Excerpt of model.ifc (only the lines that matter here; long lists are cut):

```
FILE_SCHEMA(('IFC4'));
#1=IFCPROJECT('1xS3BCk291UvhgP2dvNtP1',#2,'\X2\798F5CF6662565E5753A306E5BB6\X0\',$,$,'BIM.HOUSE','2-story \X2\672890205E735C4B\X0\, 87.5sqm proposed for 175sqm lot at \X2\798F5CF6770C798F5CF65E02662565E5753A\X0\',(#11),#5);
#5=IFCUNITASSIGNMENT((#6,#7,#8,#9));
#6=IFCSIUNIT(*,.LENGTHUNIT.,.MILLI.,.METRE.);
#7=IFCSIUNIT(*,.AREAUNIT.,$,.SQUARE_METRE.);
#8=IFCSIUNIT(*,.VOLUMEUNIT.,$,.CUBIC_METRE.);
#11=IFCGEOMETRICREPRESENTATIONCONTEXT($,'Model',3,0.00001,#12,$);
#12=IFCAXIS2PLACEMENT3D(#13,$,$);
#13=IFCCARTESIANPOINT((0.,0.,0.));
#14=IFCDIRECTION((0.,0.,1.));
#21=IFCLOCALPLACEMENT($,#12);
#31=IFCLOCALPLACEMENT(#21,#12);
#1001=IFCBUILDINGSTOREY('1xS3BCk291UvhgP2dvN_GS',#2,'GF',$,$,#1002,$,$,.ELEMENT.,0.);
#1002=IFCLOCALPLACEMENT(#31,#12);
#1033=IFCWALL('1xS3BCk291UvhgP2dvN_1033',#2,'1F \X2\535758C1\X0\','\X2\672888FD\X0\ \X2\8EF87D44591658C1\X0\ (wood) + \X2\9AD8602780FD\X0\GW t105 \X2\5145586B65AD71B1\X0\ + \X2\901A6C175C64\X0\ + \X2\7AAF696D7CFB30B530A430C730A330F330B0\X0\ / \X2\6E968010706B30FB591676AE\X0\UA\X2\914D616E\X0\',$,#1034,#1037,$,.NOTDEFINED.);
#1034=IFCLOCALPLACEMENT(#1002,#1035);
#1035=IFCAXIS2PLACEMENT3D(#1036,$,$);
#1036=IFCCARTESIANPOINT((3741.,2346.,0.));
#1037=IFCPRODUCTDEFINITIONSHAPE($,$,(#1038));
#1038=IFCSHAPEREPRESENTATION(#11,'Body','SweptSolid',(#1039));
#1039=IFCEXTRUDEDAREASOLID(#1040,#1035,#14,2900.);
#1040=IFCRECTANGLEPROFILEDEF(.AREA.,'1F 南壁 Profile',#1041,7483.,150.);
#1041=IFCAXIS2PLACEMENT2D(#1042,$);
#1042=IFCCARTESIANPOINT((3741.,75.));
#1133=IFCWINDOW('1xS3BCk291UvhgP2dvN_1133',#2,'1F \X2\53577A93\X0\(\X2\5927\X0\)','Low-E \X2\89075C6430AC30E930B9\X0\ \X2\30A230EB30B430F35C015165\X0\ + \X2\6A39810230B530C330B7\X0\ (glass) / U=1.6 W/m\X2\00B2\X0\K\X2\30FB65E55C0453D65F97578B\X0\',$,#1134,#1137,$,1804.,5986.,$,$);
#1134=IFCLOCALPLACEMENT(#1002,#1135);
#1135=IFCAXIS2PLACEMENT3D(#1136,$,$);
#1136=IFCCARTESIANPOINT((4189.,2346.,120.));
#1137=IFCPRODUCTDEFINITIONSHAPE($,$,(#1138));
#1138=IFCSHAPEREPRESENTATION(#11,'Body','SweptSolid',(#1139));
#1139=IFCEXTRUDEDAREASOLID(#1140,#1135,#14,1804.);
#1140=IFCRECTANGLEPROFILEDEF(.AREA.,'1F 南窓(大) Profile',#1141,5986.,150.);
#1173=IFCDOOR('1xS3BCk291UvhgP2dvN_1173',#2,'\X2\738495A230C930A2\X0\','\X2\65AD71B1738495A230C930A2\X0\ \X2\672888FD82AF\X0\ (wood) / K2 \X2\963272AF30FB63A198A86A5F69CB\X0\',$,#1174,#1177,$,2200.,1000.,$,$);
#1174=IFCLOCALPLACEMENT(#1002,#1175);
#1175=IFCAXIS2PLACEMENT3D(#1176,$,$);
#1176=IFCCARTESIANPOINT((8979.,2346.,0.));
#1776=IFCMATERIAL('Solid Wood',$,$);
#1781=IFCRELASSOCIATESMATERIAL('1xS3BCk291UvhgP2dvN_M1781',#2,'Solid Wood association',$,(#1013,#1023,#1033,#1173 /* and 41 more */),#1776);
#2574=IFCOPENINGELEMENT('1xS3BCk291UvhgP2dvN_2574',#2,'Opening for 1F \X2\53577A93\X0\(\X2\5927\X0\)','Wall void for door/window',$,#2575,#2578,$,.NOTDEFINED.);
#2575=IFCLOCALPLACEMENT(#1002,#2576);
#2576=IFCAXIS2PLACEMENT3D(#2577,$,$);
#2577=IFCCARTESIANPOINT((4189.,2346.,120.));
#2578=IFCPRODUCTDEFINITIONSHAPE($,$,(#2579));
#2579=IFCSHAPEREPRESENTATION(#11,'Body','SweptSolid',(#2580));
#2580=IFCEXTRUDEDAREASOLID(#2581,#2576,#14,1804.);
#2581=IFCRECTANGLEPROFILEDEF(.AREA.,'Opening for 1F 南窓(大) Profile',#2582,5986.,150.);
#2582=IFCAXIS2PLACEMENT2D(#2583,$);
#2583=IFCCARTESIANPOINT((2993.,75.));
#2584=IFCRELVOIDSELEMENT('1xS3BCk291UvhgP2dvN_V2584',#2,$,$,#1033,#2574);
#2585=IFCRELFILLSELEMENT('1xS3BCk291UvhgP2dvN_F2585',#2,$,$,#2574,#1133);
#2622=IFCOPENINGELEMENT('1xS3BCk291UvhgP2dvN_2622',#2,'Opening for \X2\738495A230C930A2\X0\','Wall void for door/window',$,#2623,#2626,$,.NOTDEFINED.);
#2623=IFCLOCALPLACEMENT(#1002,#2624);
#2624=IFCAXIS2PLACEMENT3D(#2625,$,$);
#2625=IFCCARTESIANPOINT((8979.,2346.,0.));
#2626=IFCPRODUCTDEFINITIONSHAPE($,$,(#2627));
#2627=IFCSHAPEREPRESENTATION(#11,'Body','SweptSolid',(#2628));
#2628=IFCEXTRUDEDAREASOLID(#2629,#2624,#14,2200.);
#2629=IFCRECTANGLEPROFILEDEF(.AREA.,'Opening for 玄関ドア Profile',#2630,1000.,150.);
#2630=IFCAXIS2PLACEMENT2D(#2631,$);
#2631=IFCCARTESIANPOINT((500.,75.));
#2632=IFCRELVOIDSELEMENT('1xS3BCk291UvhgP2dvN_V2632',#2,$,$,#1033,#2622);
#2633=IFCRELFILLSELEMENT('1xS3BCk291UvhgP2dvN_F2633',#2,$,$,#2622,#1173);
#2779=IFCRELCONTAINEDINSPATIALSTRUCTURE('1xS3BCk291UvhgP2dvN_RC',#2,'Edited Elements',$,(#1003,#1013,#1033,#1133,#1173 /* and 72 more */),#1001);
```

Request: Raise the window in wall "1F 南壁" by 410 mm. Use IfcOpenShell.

```python
import numpy as np
import ifcopenshell
import ifcopenshell.api.geometry
import ifcopenshell.util.placement
import ifcopenshell.util.unit

model = ifcopenshell.open("model.ifc")
unit_scale = ifcopenshell.util.unit.calculate_unit_scale(model)

window = model.by_id(1133)
opening = window.FillsVoids[0].RelatingOpeningElement
dz = 0.41 / unit_scale

shift = np.array([0.0, 0.0, dz])
# The window is not placed relative to its opening, so move both.
for product in (opening, window):
    matrix = ifcopenshell.util.placement.get_local_placement(product.ObjectPlacement)
    matrix[:3, 3] += shift
    ifcopenshell.api.geometry.edit_object_placement(model, product=product, matrix=matrix, is_si=False)

print(f"moved by {dz * unit_scale:+.3f} m")

model.write("model_updated.ifc")
```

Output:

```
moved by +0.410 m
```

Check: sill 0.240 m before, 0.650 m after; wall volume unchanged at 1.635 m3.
